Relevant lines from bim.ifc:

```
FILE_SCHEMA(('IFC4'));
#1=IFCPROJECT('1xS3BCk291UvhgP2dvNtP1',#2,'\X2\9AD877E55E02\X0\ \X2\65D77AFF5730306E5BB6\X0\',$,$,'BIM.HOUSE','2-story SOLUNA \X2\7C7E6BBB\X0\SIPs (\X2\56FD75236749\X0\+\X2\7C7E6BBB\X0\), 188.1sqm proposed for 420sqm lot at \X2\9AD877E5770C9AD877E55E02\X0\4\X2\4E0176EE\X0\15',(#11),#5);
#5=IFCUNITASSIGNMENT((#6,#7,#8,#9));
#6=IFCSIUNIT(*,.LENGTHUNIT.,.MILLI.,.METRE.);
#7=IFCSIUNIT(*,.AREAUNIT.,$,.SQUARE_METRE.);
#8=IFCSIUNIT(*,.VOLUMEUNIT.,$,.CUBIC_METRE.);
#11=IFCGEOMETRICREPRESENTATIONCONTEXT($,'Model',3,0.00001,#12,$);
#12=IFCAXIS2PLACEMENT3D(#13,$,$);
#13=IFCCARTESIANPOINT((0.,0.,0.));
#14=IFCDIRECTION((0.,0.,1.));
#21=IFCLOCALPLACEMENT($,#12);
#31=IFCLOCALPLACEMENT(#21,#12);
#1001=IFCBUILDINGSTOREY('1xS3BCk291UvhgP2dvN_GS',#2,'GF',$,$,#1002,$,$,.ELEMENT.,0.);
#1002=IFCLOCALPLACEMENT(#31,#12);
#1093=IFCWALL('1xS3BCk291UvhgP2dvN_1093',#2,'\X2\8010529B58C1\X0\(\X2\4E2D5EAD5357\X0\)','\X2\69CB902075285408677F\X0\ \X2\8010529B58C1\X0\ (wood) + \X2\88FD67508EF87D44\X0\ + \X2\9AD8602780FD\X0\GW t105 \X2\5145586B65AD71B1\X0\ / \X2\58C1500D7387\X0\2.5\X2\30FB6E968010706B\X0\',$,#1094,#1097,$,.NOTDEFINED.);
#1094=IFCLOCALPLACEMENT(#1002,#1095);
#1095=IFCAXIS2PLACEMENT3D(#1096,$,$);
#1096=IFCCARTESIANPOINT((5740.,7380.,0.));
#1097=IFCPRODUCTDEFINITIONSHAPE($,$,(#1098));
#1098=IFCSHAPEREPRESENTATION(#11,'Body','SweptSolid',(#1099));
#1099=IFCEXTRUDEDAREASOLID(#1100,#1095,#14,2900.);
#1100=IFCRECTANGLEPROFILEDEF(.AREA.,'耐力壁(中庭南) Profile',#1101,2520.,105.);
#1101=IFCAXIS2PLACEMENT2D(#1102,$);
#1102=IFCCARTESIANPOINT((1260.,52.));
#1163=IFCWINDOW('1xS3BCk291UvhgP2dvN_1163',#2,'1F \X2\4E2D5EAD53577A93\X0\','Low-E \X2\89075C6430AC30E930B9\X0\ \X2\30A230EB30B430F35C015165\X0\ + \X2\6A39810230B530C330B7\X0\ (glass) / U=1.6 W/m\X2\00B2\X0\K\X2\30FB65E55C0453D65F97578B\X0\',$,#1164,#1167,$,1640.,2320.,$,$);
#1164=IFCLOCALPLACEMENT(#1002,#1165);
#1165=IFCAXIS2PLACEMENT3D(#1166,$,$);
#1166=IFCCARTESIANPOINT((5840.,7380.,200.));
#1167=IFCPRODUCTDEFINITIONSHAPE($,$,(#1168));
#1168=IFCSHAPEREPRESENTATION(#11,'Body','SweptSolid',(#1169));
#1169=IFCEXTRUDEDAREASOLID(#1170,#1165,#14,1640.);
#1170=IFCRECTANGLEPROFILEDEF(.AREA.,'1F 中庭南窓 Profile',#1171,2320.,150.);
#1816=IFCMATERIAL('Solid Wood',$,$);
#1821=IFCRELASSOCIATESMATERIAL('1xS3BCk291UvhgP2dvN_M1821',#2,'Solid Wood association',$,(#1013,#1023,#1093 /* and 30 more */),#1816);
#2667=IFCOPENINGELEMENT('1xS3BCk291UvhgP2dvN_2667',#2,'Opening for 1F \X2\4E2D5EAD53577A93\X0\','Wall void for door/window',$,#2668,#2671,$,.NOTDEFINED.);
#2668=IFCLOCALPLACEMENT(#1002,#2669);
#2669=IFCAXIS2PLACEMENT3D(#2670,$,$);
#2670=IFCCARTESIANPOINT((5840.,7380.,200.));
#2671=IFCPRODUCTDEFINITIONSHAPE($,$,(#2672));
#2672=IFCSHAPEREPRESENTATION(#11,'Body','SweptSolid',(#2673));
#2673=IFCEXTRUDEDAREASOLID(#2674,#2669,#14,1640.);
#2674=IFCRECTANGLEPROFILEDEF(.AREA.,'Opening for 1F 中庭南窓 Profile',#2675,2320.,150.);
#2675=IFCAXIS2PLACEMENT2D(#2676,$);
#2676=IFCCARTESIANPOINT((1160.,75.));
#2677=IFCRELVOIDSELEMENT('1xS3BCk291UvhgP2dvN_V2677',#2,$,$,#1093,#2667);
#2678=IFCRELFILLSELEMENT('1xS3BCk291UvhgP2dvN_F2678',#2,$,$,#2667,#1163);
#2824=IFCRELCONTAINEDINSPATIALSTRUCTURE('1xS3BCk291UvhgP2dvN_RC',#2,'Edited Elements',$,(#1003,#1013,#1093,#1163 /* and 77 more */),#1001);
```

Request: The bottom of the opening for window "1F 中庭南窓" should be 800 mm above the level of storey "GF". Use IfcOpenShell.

```python
import numpy as np
import ifcopenshell
import ifcopenshell.api.geometry
import ifcopenshell.geom
import ifcopenshell.util.element
import ifcopenshell.util.placement
import ifcopenshell.util.shape
import ifcopenshell.util.unit

model = ifcopenshell.open("bim.ifc")
unit_scale = ifcopenshell.util.unit.calculate_unit_scale(model)

window = model.by_guid("1xS3BCk291UvhgP2dvN_1163")
opening = window.FillsVoids[0].RelatingOpeningElement
storey = ifcopenshell.util.element.get_container(window, ifc_class="IfcBuildingStorey")
level = ifcopenshell.util.placement.get_local_placement(storey.ObjectPlacement)[2, 3]

# The opening's origin need not be at the sill, so measure its lowest point.
shape = ifcopenshell.geom.create_shape(ifcopenshell.geom.settings(), opening)
bottom = ifcopenshell.util.shape.get_shape_bottom_elevation(shape, shape.geometry) / unit_scale
dz = level + 0.8 / unit_scale - bottom

shift = np.array([0.0, 0.0, dz])
# The window is not placed relative to its opening, so move both.
for product in (opening, window):
    matrix = ifcopenshell.util.placement.get_local_placement(product.ObjectPlacement)
    matrix[:3, 3] += shift
    ifcopenshell.api.geometry.edit_object_placement(model, product=product, matrix=matrix, is_si=False)

print(f"moved by {dz * unit_scale:+.3f} m")

model.write("bim_v2.ifc")
```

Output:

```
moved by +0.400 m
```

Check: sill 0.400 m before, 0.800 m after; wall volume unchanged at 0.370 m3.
